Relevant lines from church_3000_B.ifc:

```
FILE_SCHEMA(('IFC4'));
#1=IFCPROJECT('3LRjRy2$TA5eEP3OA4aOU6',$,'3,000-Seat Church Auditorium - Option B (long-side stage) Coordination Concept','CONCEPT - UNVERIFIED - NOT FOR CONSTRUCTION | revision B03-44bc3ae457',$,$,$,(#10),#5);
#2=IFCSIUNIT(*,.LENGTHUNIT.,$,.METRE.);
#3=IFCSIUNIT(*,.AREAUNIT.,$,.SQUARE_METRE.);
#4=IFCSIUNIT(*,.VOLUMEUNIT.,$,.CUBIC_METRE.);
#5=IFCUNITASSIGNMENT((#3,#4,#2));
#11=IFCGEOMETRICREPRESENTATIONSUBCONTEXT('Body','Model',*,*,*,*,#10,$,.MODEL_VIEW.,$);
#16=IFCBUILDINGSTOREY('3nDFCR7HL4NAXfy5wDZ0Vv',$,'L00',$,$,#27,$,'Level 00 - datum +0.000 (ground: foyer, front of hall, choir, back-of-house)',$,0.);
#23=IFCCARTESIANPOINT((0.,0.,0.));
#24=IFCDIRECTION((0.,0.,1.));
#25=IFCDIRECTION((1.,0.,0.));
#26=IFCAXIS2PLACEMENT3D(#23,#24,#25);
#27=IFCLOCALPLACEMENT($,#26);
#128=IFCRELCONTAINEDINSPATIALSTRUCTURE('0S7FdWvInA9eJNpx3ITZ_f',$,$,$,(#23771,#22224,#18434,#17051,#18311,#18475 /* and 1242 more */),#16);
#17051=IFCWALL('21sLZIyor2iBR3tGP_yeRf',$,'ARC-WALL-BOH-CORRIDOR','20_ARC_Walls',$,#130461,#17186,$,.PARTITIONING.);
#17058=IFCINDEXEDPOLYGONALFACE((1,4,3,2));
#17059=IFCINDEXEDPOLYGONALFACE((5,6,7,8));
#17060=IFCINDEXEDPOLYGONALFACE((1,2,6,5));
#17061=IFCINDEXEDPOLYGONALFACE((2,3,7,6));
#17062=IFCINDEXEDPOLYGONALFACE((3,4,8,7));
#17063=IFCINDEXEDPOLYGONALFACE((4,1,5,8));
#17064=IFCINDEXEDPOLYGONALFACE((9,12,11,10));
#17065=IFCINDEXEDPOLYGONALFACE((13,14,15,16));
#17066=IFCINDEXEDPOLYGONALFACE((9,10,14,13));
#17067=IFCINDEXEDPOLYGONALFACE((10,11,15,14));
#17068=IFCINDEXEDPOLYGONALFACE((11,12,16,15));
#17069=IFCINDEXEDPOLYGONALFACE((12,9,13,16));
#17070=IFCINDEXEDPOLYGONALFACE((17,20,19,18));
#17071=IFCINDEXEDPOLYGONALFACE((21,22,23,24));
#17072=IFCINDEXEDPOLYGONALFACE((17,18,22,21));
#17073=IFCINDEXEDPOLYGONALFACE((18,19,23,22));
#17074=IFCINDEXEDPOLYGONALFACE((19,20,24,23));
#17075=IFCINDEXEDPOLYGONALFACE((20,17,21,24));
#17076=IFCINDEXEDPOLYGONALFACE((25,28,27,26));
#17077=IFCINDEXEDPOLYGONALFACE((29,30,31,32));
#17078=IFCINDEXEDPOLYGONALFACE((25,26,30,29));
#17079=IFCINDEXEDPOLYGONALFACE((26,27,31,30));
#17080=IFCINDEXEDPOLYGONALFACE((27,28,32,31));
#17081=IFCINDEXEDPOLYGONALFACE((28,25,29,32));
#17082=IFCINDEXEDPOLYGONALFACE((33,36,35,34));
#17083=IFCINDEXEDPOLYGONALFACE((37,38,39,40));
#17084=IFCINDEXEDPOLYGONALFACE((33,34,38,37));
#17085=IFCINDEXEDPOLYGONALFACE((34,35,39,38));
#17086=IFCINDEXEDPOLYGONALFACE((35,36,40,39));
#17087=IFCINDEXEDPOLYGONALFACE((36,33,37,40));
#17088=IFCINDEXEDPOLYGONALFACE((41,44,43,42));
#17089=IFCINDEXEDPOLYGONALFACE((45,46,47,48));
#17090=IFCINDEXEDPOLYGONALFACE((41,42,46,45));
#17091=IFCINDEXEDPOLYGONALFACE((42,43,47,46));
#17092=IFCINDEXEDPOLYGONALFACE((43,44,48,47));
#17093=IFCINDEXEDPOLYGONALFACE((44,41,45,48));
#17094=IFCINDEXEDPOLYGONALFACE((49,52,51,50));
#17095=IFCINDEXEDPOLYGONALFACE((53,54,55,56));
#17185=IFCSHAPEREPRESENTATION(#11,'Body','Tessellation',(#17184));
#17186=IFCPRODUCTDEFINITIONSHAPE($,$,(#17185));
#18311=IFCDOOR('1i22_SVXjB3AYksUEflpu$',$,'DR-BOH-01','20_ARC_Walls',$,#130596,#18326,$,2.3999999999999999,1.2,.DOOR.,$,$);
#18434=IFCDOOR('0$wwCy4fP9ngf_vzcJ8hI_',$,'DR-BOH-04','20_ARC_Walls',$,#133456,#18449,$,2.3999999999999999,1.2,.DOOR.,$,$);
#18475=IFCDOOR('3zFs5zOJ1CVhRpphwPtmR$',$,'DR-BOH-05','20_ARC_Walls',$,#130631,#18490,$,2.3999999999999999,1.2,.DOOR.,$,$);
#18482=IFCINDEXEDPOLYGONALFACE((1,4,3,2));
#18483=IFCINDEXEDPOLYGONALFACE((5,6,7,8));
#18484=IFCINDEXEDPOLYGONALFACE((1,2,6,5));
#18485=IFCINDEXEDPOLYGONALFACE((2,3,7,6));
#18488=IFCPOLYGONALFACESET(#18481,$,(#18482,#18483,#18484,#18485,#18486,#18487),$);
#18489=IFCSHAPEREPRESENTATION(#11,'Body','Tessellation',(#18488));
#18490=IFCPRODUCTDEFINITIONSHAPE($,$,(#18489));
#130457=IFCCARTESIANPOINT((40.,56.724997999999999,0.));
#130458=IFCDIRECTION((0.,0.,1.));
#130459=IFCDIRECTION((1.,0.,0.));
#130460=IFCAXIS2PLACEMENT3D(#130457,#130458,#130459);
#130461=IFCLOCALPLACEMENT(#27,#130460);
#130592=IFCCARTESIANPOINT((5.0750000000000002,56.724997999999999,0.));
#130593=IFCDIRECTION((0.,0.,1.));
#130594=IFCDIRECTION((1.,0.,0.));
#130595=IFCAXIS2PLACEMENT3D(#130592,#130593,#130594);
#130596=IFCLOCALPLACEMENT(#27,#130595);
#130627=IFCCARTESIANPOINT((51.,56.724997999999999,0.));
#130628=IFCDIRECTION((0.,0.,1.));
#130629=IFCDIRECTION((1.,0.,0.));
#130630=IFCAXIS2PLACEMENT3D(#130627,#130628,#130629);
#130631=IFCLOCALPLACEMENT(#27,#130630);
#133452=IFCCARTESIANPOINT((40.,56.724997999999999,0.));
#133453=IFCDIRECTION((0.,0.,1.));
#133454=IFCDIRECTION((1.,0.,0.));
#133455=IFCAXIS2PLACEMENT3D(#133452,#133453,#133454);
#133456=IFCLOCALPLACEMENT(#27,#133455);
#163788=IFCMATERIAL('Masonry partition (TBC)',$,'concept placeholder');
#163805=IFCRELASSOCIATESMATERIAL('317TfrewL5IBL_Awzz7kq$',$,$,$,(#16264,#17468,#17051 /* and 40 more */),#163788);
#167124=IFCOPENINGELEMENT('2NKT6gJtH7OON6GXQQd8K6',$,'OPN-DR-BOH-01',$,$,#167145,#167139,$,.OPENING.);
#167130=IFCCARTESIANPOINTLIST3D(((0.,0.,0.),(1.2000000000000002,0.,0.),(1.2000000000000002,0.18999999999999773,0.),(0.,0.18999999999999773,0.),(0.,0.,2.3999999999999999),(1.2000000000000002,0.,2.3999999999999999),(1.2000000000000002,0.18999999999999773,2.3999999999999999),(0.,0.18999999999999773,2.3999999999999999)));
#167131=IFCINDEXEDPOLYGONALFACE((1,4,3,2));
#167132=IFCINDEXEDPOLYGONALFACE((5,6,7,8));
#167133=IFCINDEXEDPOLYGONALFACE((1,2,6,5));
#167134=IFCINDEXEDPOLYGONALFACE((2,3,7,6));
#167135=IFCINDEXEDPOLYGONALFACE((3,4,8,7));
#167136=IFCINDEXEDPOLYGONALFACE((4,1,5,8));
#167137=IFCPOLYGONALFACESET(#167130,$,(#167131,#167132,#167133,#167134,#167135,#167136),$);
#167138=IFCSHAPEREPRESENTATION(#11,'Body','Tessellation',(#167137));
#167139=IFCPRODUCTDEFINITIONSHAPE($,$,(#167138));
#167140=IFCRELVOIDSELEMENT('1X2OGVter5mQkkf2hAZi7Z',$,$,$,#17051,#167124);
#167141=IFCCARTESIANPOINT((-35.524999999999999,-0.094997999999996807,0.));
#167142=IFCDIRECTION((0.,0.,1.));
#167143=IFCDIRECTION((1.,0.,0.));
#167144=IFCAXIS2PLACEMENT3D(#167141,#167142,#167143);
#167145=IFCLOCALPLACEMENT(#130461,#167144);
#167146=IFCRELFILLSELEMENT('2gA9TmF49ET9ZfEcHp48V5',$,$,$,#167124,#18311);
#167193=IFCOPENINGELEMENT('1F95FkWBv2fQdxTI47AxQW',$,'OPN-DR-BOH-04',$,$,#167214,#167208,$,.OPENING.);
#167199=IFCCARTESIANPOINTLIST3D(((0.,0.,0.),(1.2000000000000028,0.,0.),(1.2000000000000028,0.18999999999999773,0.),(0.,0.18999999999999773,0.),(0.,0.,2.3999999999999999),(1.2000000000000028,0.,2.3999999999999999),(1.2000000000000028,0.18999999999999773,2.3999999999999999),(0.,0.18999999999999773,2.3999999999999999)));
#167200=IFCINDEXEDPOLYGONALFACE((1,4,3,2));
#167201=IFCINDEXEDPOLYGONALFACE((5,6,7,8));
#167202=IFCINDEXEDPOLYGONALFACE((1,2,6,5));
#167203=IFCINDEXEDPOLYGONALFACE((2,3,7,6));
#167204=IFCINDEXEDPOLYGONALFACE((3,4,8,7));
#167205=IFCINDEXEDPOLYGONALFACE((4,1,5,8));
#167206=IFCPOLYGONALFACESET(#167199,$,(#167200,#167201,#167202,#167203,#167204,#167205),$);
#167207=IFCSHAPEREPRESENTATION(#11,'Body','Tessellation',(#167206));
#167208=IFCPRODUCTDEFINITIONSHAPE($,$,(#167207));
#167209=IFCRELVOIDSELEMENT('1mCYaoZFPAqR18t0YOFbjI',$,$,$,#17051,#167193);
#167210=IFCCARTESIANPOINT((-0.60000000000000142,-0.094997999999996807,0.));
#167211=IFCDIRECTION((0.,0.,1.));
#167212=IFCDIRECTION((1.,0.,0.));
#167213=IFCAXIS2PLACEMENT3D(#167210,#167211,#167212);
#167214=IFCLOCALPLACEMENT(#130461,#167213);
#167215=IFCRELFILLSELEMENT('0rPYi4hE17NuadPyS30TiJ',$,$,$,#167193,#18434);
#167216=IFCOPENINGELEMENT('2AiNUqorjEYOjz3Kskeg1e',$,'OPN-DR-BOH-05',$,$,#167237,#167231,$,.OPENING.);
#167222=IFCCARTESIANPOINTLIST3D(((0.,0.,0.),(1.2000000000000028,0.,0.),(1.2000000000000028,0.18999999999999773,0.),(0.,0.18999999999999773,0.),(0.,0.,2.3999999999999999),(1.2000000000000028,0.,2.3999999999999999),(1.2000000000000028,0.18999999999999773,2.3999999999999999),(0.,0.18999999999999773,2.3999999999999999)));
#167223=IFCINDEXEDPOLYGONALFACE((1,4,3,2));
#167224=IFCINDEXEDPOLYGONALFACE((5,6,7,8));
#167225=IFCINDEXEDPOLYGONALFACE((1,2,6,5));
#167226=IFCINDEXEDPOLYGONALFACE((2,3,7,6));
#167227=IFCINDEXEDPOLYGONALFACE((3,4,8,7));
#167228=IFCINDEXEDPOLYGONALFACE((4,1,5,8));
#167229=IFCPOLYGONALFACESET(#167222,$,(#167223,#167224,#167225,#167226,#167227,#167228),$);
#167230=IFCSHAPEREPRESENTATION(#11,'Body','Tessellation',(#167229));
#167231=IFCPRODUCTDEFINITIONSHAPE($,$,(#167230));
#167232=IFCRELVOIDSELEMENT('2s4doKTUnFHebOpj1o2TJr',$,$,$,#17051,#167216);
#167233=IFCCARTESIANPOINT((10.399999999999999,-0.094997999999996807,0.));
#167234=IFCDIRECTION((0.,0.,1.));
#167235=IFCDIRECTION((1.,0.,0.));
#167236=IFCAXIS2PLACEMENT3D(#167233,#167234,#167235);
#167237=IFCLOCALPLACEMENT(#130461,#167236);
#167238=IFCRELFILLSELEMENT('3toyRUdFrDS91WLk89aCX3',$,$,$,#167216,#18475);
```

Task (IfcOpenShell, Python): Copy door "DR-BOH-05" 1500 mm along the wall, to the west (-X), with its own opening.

```python
import ifcopenshell
import ifcopenshell.api.feature
import ifcopenshell.api.geometry
import ifcopenshell.api.root
import ifcopenshell.geom
import ifcopenshell.util.element
import ifcopenshell.util.placement
import ifcopenshell.util.shape

model = ifcopenshell.open("church_3000_B.ifc")
settings = ifcopenshell.geom.settings()


def volume(element):
    """Net volume in cubic metres, openings subtracted."""
    shape = ifcopenshell.geom.create_shape(settings, element)
    return ifcopenshell.util.shape.get_volume(shape.geometry)


door = model.by_id(18475)
opening = door.FillsVoids[0].RelatingOpeningElement
wall = opening.VoidsElements[0].RelatingBuildingElement
before = volume(wall)
shift = ifcopenshell.util.placement.get_local_placement(wall.ObjectPlacement)[:3, 0] * -1.5

# copy_class copies the void relationship, type, container and properties, but no geometry.
new_opening = ifcopenshell.api.root.copy_class(model, product=opening)
new_opening.Representation = ifcopenshell.util.element.copy_deep(
    model, opening.Representation, exclude=["IfcGeometricRepresentationContext", "IfcRepresentationMap"]
)
new_door = ifcopenshell.api.root.copy_class(model, product=door)
new_door.Representation = ifcopenshell.util.element.copy_deep(
    model, door.Representation, exclude=["IfcGeometricRepresentationContext", "IfcRepresentationMap"]
)
ifcopenshell.api.feature.add_filling(model, opening=new_opening, element=new_door)

for old, new in ((opening, new_opening), (door, new_door)):
    matrix = ifcopenshell.util.placement.get_local_placement(old.ObjectPlacement)
    matrix[:3, 3] += shift
    ifcopenshell.api.geometry.edit_object_placement(model, product=new, matrix=matrix, is_si=False)

after = volume(wall)

print(f"wall volume {before:.3f} -> {after:.3f} m3")

model.write("church_3000_B_updated.ifc")
```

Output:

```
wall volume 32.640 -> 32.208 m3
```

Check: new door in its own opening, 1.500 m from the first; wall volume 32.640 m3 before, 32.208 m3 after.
